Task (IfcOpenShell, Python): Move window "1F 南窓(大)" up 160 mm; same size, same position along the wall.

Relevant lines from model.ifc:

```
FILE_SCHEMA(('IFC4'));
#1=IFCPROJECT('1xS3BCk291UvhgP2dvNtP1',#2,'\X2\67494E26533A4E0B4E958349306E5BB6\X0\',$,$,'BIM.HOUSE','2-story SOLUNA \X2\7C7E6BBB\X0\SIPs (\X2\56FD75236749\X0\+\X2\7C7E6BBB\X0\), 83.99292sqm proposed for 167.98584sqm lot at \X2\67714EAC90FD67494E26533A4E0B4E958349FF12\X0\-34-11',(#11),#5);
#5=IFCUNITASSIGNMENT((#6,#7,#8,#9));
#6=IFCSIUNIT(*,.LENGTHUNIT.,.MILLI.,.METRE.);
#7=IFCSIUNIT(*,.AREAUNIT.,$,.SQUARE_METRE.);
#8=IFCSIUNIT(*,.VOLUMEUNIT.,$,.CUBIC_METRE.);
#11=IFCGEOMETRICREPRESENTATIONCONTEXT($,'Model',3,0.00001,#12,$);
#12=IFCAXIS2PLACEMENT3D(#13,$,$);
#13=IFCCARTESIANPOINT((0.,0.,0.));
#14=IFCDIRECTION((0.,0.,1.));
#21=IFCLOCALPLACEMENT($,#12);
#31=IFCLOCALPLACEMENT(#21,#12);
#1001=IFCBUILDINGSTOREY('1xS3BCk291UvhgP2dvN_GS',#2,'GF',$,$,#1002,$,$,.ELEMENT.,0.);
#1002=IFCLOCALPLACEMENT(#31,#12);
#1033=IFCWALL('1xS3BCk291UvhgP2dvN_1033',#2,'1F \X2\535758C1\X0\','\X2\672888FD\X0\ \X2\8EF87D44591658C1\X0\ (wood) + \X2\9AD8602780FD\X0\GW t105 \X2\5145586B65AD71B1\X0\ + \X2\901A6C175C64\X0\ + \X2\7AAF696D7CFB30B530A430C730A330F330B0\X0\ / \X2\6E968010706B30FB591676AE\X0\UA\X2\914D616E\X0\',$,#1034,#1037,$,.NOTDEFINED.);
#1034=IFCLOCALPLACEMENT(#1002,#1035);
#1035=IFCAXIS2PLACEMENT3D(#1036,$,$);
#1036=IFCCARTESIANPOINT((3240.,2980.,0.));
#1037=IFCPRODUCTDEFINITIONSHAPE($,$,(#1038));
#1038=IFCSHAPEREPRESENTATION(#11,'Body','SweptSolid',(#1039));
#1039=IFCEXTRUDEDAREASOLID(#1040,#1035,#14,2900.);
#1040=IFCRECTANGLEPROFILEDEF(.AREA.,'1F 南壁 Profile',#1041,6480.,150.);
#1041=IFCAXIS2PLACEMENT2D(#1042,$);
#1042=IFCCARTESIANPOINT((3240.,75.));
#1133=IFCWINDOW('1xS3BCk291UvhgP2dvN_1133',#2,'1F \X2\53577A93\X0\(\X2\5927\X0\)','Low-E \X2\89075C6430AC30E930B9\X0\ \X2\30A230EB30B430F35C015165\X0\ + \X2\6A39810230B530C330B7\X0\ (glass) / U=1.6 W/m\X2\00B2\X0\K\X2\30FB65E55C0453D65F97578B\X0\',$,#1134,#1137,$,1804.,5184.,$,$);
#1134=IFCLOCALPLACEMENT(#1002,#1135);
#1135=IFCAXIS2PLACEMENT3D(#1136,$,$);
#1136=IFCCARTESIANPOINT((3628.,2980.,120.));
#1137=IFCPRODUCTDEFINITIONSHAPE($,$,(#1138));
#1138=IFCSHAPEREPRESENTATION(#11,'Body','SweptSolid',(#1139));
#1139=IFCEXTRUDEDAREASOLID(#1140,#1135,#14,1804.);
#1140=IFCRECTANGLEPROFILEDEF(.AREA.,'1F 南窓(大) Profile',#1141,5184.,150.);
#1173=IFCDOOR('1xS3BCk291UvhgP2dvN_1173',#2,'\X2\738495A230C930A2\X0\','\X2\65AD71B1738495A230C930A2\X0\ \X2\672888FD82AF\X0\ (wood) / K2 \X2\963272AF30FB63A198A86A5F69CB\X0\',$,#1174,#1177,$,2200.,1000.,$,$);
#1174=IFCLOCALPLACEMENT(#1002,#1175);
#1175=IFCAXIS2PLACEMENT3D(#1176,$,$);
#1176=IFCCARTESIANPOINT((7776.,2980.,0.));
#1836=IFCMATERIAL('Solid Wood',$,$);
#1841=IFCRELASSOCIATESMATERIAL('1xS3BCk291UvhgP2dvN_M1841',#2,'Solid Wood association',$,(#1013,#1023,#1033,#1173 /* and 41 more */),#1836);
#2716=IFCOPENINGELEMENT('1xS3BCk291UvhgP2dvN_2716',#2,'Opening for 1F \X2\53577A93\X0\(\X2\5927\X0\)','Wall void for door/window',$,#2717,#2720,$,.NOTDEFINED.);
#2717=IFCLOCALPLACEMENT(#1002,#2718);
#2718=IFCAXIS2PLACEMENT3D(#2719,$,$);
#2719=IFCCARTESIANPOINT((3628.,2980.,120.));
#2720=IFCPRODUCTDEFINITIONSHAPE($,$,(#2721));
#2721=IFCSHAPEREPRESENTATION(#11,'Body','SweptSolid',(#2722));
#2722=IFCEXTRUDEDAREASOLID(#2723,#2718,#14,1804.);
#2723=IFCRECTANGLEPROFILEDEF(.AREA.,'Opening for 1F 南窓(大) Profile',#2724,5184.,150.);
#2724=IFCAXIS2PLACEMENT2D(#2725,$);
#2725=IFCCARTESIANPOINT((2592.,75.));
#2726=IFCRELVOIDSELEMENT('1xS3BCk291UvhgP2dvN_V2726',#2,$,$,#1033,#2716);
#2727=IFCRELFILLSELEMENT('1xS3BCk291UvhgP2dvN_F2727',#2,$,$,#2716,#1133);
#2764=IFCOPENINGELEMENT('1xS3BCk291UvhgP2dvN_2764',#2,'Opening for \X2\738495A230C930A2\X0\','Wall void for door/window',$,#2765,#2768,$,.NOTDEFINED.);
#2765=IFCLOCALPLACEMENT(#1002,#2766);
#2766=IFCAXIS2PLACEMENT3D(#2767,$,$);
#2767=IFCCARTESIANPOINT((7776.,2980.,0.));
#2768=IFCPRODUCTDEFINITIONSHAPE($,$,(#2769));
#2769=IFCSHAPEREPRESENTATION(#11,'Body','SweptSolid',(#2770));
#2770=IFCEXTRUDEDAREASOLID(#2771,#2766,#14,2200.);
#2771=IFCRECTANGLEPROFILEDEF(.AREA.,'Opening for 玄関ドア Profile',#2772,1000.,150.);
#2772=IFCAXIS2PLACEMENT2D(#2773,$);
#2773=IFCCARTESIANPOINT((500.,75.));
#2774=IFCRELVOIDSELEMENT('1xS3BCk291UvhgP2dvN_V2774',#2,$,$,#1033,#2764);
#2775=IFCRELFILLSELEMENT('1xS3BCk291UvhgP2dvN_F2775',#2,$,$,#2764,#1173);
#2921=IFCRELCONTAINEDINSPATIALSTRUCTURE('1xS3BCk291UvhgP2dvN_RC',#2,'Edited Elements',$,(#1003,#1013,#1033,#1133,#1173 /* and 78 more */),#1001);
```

```python
import numpy as np
import ifcopenshell
import ifcopenshell.api.geometry
import ifcopenshell.util.placement
import ifcopenshell.util.unit

model = ifcopenshell.open("model.ifc")
unit_scale = ifcopenshell.util.unit.calculate_unit_scale(model)

window = model.by_id(1133)
opening = window.FillsVoids[0].RelatingOpeningElement
dz = 160.0

shift = np.array([0.0, 0.0, dz])
# The window is not placed relative to its opening, so move both.
for product in (opening, window):
    matrix = ifcopenshell.util.placement.get_local_placement(product.ObjectPlacement)
    matrix[:3, 3] += shift
    ifcopenshell.api.geometry.edit_object_placement(model, product=product, matrix=matrix, is_si=False)

print(f"moved by {dz * unit_scale:+.3f} m")

model.write("model_edited.ifc")
```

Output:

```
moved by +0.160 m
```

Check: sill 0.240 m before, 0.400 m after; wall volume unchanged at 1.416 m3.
